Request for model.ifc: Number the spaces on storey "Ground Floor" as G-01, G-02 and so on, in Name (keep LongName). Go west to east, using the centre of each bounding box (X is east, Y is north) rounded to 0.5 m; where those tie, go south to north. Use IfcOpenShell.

First a look at what the model holds.

```python
import ifcopenshell
import ifcopenshell.util.element
import ifcopenshell.util.placement

model = ifcopenshell.open("model.ifc")
print(model.schema)
storey = next(s for s in model.by_type("IfcBuildingStorey") if s.Name == "Ground Floor")
spaces = [e for e in ifcopenshell.util.element.get_decomposition(storey) if e.is_a("IfcSpace")]
for e in sorted(spaces, key=lambda e: e.id()):
    origin = ifcopenshell.util.placement.get_local_placement(e.ObjectPlacement)[:3, 3]
    print(e.id(), e.Name, e.LongName, origin.round(2) + 0.0, sep=" | ")
```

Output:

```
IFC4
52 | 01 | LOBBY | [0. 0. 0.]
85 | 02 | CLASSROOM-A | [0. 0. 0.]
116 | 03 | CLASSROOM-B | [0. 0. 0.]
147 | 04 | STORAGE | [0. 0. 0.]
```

```python
import ifcopenshell
import ifcopenshell.geom
import ifcopenshell.util.element
import ifcopenshell.util.shape

model = ifcopenshell.open("model.ifc")
settings = ifcopenshell.geom.settings()
settings.set("use-world-coords", True)


def centre(element):
    shape = ifcopenshell.geom.create_shape(settings, element)
    return ifcopenshell.util.shape.get_bbox_centroid(shape.geometry)


storey = next(s for s in model.by_type("IfcBuildingStorey") if s.Name == "Ground Floor")
spaces = [e for e in ifcopenshell.util.element.get_decomposition(storey) if e.is_a("IfcSpace")]

# Insertion points can sit at a corner or the storey origin, so sort by the geometry (in metres).
centres = {e: centre(e) for e in spaces}
spaces.sort(key=lambda e: (round(centres[e][0] / 0.5), centres[e][1]))

for i, e in enumerate(spaces, start=1):
    number = f"G-{i:02d}"
    e.Name = number
    print(e.id(), number)

model.write("model_rev.ifc")
```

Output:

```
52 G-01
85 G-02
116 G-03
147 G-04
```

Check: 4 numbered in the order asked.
